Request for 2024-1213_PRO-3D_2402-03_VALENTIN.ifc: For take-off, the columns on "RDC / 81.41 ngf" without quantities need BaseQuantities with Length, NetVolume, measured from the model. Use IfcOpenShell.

First a look at what the model holds.

```python
import ifcopenshell
import ifcopenshell.util.element
import ifcopenshell.util.unit

model = ifcopenshell.open("2024-1213_PRO-3D_2402-03_VALENTIN.ifc")
print(model.schema)
for unit_type in ("LENGTHUNIT", "AREAUNIT", "VOLUMEUNIT"):
    print(unit_type, ifcopenshell.util.unit.calculate_unit_scale(model, unit_type))
storey = next(s for s in model.by_type("IfcBuildingStorey") if s.Name == "RDC / 81.41 ngf")
columns = [e for e in ifcopenshell.util.element.get_decomposition(storey) if e.is_a("IfcColumn")]
for e in sorted(columns, key=lambda e: e.id()):
    print(e.id(), e.is_a(), e.Name, list(ifcopenshell.util.element.get_psets(e, qtos_only=True)), sep=" | ")
```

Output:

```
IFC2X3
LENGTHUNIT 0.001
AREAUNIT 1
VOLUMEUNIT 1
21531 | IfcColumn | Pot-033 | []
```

```python
import ifcopenshell
import ifcopenshell.api.pset
import ifcopenshell.geom
import ifcopenshell.util.element
import ifcopenshell.util.shape
import ifcopenshell.util.unit

model = ifcopenshell.open("2024-1213_PRO-3D_2402-03_VALENTIN.ifc")
unit_scale = ifcopenshell.util.unit.calculate_unit_scale(model)
volume_scale = ifcopenshell.util.unit.calculate_unit_scale(model, "VOLUMEUNIT")
settings = ifcopenshell.geom.settings()

storey = next(s for s in model.by_type("IfcBuildingStorey") if s.Name == "RDC / 81.41 ngf")
columns = [e for e in ifcopenshell.util.element.get_decomposition(storey) if e.is_a("IfcColumn")]

for e in sorted(columns, key=lambda e: e.id()):
    if ifcopenshell.util.element.get_psets(e, qtos_only=True, should_inherit=False):
        continue
    # Geometry comes back in metres, in the element's own axes.
    shape = ifcopenshell.geom.create_shape(settings, e)
    values = {
        "Length": ifcopenshell.util.shape.get_z(shape.geometry) / unit_scale,
        "NetVolume": ifcopenshell.util.shape.get_volume(shape.geometry) / volume_scale,
    }
    qto = ifcopenshell.api.pset.add_qto(model, product=e, name="BaseQuantities")
    ifcopenshell.api.pset.edit_qto(model, qto=qto, properties=values)
    print(e.id(), {k: round(v, 3) for k, v in values.items()})

model.write("2024-1213_PRO-3D_2402-03_VALENTIN_updated.ifc")
```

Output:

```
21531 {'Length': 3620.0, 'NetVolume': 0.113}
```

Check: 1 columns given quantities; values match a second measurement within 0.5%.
